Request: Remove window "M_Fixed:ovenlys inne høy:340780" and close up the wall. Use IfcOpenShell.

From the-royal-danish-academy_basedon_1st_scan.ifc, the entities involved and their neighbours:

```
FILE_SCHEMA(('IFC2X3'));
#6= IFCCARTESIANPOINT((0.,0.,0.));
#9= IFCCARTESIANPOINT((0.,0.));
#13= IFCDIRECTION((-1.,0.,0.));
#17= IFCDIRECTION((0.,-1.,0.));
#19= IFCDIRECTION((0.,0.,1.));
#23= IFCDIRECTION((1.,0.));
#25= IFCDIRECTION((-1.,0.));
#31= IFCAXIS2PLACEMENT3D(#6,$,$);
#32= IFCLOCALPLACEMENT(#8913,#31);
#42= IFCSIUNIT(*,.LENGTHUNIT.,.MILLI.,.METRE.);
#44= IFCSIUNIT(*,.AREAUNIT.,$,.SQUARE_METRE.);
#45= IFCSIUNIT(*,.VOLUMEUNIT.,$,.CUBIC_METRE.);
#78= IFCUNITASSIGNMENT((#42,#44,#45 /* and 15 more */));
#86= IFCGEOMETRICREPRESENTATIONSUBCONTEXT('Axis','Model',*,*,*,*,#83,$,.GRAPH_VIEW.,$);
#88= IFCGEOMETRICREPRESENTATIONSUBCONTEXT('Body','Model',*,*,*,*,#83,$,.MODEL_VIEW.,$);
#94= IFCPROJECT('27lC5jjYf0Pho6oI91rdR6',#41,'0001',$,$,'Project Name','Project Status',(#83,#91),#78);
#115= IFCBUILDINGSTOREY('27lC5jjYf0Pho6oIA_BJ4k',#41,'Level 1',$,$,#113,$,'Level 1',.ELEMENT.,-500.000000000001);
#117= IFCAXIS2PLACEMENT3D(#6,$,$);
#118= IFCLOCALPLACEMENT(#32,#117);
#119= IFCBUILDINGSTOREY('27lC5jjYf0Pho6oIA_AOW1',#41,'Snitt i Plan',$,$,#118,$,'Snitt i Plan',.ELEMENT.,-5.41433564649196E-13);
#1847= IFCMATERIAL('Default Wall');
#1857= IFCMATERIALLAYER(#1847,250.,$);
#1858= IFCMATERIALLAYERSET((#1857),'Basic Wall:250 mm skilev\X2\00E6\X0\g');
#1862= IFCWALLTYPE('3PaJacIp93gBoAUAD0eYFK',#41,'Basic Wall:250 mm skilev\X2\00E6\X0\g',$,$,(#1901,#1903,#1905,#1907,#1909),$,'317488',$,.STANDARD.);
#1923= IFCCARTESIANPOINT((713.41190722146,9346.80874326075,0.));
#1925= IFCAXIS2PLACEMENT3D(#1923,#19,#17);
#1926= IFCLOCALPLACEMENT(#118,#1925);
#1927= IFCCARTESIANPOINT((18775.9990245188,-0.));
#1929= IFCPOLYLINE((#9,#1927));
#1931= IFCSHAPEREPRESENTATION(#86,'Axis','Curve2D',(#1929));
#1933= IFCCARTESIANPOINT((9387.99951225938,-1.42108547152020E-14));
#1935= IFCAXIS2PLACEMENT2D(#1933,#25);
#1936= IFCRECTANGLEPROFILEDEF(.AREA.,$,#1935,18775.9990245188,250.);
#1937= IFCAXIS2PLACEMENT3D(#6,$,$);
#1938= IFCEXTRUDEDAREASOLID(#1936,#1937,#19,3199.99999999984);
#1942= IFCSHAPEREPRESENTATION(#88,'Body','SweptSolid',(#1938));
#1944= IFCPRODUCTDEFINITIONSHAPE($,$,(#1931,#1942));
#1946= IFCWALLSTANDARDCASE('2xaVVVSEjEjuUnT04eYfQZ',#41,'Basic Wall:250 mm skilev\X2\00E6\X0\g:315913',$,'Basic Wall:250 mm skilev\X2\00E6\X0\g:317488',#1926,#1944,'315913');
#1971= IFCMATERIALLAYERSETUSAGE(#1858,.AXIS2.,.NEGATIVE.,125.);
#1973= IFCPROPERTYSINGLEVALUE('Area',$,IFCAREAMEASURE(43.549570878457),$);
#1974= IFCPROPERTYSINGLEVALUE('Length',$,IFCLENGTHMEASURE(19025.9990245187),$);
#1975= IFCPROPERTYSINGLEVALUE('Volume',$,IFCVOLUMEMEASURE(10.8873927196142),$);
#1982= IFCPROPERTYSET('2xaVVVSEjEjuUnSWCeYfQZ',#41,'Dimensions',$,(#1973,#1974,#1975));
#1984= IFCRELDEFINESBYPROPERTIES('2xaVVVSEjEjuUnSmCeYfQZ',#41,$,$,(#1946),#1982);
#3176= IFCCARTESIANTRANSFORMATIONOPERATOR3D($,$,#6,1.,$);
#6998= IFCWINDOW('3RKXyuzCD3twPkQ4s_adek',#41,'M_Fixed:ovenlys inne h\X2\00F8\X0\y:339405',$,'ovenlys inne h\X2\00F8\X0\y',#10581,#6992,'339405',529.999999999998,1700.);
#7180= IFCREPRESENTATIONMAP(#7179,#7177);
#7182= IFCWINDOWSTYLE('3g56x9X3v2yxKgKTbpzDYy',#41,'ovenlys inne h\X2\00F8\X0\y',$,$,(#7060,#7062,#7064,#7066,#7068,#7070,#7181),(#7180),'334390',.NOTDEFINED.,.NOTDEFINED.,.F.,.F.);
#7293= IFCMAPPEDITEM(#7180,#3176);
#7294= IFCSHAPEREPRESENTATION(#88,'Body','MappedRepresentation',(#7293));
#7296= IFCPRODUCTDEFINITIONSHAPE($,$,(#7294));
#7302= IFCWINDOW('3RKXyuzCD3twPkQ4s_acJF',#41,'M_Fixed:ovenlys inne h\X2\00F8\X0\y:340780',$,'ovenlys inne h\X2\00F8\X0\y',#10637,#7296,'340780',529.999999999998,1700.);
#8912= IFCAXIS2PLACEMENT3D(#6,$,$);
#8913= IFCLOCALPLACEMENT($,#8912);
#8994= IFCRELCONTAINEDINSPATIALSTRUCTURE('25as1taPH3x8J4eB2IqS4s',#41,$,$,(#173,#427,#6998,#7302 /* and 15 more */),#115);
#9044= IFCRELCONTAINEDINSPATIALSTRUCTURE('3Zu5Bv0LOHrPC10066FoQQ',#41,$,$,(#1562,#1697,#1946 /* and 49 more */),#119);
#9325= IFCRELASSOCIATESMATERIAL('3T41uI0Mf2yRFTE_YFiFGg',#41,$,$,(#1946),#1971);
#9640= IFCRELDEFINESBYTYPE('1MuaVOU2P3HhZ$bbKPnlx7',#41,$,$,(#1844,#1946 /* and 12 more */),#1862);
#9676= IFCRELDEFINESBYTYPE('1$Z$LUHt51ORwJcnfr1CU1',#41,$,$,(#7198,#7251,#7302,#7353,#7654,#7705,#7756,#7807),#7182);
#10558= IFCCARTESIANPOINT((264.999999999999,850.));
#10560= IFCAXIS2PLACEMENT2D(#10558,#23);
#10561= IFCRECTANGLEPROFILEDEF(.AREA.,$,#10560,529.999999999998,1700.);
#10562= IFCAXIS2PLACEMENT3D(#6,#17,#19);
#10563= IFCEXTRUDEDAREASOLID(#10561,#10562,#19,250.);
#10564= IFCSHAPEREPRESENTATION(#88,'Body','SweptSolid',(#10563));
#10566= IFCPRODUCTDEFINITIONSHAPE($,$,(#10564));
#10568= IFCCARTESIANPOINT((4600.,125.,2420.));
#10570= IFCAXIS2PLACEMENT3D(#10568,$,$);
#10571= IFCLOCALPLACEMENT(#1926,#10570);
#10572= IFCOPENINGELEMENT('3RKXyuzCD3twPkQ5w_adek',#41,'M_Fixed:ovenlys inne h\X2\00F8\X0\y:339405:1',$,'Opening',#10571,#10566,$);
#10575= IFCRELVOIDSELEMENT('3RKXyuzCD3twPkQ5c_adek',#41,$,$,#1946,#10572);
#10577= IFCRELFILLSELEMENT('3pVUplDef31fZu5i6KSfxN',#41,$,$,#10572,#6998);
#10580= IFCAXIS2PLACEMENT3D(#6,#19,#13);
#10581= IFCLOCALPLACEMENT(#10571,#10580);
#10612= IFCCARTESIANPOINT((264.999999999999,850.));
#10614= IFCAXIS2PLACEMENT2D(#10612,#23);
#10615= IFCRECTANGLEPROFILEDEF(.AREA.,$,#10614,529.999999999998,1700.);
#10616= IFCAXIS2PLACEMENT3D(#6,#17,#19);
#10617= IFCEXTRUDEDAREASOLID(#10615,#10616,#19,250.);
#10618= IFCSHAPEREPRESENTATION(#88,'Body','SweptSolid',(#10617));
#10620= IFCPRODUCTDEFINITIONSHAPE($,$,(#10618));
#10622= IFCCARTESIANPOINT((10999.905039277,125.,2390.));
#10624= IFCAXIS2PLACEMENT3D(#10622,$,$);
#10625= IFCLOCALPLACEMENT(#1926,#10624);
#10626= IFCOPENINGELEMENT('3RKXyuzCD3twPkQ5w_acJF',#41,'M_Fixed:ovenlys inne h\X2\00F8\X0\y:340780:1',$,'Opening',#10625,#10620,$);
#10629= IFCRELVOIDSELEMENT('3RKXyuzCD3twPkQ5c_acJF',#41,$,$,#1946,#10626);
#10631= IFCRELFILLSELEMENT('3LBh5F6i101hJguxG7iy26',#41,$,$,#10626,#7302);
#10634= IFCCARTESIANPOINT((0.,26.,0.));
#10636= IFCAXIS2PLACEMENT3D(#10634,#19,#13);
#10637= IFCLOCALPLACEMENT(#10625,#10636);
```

```python
import ifcopenshell
import ifcopenshell.api.feature
import ifcopenshell.api.pset
import ifcopenshell.api.root
import ifcopenshell.geom
import ifcopenshell.util.element
import ifcopenshell.util.shape
import ifcopenshell.util.unit

model = ifcopenshell.open("the-royal-danish-academy_basedon_1st_scan.ifc")
area_scale = ifcopenshell.util.unit.calculate_unit_scale(model, "AREAUNIT")
volume_scale = ifcopenshell.util.unit.calculate_unit_scale(model, "VOLUMEUNIT")
settings = ifcopenshell.geom.settings()


def volume(element):
    """Net volume in cubic metres, openings subtracted."""
    shape = ifcopenshell.geom.create_shape(settings, element)
    return ifcopenshell.util.shape.get_volume(shape.geometry)


window = model.by_guid("3RKXyuzCD3twPkQ4s_acJF")
opening = window.FillsVoids[0].RelatingOpeningElement
wall = opening.VoidsElements[0].RelatingBuildingElement
before = volume(wall)

ifcopenshell.api.root.remove_product(model, product=window)
ifcopenshell.api.feature.remove_feature(model, feature=opening)

after = volume(wall)
thickness = 0.25  # wall thickness in metres

# Update the wall's stored quantities.
pset = model.by_id(ifcopenshell.util.element.get_pset(wall, "Dimensions", should_inherit=False)["id"])
ifcopenshell.api.pset.edit_pset(model, pset=pset, properties={
    "Area": model.create_entity("IfcAreaMeasure", after / thickness / area_scale),
    "Volume": model.create_entity("IfcVolumeMeasure", after / volume_scale),
})

print(f"wall volume {before:.3f} -> {after:.3f} m3")

model.write("the-royal-danish-academy_basedon_1st_scan_v2.ifc")
```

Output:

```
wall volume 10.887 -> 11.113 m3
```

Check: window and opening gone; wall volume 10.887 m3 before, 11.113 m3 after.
